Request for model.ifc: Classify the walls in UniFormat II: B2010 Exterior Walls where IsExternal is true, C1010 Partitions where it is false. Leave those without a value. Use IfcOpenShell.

First a look at what the model holds.

```python
import ifcopenshell
import ifcopenshell.util.element

model = ifcopenshell.open("model.ifc")
print(model.schema)
print("classifications:", [c.Name for c in model.by_type("IfcClassification")])
values = [ifcopenshell.util.element.get_pset(e, "Pset_WallCommon", "IsExternal") for e in model.by_type("IfcWall")]
for value in (True, False, None):
    print("IsExternal", value, values.count(value))
```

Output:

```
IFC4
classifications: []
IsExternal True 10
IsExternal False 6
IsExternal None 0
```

```python
import ifcopenshell
import ifcopenshell.api.classification
import ifcopenshell.util.element

model = ifcopenshell.open("model.ifc")

system = ifcopenshell.api.classification.add_classification(model, classification="UniFormat II")

walls = model.by_type("IfcWall")
external = {e: ifcopenshell.util.element.get_pset(e, "Pset_WallCommon", "IsExternal") for e in walls}
for flag, code, name in ((True, "B2010", "Exterior Walls"), (False, "C1010", "Partitions")):
    products = [e for e in walls if external[e] is flag]
    ifcopenshell.api.classification.add_reference(
        model, products=products, classification=system, identification=code, name=name
    )
    print(code, len(products))

model.write("model_edited.ifc")
```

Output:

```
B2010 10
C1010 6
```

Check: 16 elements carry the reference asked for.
